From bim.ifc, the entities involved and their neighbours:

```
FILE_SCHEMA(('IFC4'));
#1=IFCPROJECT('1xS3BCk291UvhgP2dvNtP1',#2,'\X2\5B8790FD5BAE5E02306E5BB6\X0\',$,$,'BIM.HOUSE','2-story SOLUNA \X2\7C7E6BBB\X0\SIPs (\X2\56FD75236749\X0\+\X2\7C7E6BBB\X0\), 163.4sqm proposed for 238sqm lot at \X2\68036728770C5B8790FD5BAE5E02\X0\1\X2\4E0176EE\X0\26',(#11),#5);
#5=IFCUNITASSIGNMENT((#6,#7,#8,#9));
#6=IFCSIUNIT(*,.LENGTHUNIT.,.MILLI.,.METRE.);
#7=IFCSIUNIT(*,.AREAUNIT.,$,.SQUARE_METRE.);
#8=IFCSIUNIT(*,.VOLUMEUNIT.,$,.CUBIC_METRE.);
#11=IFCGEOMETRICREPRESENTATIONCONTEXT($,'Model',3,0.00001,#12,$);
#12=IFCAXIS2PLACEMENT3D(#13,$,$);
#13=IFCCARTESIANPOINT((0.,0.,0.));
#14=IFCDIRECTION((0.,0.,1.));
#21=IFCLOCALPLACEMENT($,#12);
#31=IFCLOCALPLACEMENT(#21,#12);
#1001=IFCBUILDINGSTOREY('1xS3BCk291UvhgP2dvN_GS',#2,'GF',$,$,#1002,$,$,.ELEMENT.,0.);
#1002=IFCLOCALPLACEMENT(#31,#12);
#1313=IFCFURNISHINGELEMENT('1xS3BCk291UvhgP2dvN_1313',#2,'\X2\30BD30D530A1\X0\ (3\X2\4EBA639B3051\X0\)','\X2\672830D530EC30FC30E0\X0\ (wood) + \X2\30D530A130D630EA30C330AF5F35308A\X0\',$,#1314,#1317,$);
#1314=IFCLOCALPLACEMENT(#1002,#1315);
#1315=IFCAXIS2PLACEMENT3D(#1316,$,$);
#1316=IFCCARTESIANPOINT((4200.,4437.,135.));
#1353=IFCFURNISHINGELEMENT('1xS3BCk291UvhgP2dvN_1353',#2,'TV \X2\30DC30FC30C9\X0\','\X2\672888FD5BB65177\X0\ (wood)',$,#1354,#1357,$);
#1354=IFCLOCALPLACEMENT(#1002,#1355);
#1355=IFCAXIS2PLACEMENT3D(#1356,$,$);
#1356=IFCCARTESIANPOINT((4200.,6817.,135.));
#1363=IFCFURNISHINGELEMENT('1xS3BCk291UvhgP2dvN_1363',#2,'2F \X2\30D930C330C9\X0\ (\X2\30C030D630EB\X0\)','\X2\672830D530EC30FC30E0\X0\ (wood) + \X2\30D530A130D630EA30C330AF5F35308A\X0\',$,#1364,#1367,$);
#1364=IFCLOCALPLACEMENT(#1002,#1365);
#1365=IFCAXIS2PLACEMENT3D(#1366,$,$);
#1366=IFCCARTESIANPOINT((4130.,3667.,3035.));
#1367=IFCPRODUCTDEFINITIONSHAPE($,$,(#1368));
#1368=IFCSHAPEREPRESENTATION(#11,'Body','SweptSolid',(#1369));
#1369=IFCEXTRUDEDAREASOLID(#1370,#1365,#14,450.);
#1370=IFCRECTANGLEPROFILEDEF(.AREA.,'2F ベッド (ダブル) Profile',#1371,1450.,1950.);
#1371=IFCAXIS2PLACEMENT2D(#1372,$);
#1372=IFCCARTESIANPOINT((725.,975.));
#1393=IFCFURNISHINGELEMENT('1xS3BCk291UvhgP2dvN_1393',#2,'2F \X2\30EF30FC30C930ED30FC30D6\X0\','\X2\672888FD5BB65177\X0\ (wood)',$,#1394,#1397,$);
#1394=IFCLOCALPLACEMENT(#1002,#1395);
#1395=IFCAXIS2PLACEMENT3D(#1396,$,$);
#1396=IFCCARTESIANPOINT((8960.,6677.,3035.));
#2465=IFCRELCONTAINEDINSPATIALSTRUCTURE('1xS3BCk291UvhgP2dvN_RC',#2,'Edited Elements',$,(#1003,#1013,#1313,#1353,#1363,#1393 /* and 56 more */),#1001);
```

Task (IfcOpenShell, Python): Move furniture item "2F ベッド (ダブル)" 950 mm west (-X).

```python
import ifcopenshell
import ifcopenshell.api.geometry
import ifcopenshell.util.placement

model = ifcopenshell.open("bim.ifc")

item = model.by_guid("1xS3BCk291UvhgP2dvN_1363")
matrix = ifcopenshell.util.placement.get_local_placement(item.ObjectPlacement)
matrix[0, 3] -= 950.0
ifcopenshell.api.geometry.edit_object_placement(model, product=item, matrix=matrix, is_si=False)

print(ifcopenshell.util.placement.get_local_placement(item.ObjectPlacement).round(3) + 0.0)

model.write("bim-out.ifc")
```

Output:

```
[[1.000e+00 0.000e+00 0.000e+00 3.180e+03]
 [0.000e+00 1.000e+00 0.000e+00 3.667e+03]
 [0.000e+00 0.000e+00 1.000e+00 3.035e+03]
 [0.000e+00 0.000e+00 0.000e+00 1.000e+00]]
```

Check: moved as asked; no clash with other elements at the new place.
